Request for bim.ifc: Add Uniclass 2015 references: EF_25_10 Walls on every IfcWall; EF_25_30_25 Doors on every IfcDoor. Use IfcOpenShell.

First a look at what the model holds.

```python
import ifcopenshell

model = ifcopenshell.open("bim.ifc")
print(model.schema)
print("classifications:", [c.Name for c in model.by_type("IfcClassification")])
for ifc_class in ("IfcDoor", "IfcRoof", "IfcStair", "IfcWall", "IfcWindow"):
    print(ifc_class, len(model.by_type(ifc_class)))
```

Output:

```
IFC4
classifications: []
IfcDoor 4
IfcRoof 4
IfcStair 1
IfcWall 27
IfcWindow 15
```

```python
import ifcopenshell
import ifcopenshell.api.classification

model = ifcopenshell.open("bim.ifc")

system = ifcopenshell.api.classification.add_classification(model, classification="Uniclass 2015")

codes = {
    "IfcWall": ("EF_25_10", "Walls"),
    "IfcDoor": ("EF_25_30_25", "Doors"),
}
for ifc_class, (code, name) in codes.items():
    products = model.by_type(ifc_class)
    ifcopenshell.api.classification.add_reference(
        model, products=products, classification=system, identification=code, name=name
    )
    print(code, len(products))

model.write("bim_updated.ifc")
```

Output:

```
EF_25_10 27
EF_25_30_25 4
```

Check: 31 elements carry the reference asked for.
